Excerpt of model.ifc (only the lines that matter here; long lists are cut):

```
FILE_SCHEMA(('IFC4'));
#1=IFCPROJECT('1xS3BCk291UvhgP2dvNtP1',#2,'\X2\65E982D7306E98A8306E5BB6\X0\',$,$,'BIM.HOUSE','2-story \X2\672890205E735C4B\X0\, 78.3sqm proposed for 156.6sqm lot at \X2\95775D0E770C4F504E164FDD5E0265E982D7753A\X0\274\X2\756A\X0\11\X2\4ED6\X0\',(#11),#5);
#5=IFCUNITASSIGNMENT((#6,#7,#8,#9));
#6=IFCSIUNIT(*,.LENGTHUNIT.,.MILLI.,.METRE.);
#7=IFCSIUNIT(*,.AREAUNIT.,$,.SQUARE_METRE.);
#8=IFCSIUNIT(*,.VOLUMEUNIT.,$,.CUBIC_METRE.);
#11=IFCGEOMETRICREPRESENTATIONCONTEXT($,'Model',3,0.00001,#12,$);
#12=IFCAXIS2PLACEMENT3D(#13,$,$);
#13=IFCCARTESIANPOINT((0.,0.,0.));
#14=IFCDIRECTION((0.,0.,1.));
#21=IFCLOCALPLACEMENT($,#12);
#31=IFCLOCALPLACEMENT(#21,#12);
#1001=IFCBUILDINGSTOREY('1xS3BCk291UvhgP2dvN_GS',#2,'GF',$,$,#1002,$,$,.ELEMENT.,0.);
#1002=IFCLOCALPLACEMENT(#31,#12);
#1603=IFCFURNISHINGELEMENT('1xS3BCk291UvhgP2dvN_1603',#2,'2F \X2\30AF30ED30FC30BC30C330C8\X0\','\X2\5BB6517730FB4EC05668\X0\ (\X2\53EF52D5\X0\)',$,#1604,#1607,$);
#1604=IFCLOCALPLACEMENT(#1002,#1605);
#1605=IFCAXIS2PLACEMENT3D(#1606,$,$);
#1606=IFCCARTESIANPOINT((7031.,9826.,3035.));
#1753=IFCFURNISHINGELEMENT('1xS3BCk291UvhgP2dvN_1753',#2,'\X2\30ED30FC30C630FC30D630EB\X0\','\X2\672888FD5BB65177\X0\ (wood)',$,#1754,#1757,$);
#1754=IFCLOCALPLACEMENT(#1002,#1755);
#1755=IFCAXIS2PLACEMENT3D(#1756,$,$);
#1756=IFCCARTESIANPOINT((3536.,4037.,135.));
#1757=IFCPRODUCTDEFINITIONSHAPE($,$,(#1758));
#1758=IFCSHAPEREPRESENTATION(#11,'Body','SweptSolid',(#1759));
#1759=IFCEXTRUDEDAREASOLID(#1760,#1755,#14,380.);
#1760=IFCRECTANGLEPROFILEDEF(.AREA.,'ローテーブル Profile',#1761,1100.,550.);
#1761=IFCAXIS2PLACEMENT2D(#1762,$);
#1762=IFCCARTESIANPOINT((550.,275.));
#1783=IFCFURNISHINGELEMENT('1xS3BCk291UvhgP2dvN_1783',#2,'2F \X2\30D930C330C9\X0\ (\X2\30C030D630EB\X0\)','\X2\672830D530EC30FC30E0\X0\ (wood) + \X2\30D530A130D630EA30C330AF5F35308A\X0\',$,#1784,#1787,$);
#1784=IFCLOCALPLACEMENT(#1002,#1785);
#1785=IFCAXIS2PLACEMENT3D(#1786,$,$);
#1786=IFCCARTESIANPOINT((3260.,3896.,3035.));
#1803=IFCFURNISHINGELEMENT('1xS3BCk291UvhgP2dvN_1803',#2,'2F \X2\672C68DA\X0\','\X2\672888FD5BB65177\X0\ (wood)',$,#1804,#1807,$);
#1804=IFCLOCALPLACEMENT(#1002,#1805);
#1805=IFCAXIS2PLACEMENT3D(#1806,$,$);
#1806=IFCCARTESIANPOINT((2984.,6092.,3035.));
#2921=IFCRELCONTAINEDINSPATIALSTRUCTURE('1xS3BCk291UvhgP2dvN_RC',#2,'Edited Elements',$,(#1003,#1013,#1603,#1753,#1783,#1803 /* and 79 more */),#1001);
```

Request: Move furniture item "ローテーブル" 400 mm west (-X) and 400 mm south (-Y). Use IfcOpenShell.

```python
import ifcopenshell
import ifcopenshell.api.geometry
import ifcopenshell.util.placement

model = ifcopenshell.open("model.ifc")

item = model.by_id(1753)
matrix = ifcopenshell.util.placement.get_local_placement(item.ObjectPlacement)
matrix[0, 3] -= 400.0
matrix[1, 3] -= 400.0
ifcopenshell.api.geometry.edit_object_placement(model, product=item, matrix=matrix, is_si=False)

print(ifcopenshell.util.placement.get_local_placement(item.ObjectPlacement).round(3) + 0.0)

model.write("model_v2.ifc")
```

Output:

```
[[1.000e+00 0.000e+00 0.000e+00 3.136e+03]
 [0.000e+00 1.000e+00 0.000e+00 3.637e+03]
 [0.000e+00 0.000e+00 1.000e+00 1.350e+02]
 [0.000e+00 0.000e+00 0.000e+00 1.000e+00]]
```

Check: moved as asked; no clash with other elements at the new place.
